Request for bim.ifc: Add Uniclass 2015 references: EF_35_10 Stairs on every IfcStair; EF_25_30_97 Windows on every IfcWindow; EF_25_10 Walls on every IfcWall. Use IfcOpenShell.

First a look at what the model holds.

```python
import ifcopenshell

model = ifcopenshell.open("bim.ifc")
print(model.schema)
print("classifications:", [c.Name for c in model.by_type("IfcClassification")])
for ifc_class in ("IfcDoor", "IfcRoof", "IfcStair", "IfcWall", "IfcWindow"):
    print(ifc_class, len(model.by_type(ifc_class)))
```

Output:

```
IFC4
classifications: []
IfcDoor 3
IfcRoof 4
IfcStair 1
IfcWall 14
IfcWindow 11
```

```python
import ifcopenshell
import ifcopenshell.api.classification

model = ifcopenshell.open("bim.ifc")

system = ifcopenshell.api.classification.add_classification(model, classification="Uniclass 2015")

codes = {
    "IfcStair": ("EF_35_10", "Stairs"),
    "IfcWindow": ("EF_25_30_97", "Windows"),
    "IfcWall": ("EF_25_10", "Walls"),
}
for ifc_class, (code, name) in codes.items():
    products = model.by_type(ifc_class)
    ifcopenshell.api.classification.add_reference(
        model, products=products, classification=system, identification=code, name=name
    )
    print(code, len(products))

model.write("bim-out.ifc")
```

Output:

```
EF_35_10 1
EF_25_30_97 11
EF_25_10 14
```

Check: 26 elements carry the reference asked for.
